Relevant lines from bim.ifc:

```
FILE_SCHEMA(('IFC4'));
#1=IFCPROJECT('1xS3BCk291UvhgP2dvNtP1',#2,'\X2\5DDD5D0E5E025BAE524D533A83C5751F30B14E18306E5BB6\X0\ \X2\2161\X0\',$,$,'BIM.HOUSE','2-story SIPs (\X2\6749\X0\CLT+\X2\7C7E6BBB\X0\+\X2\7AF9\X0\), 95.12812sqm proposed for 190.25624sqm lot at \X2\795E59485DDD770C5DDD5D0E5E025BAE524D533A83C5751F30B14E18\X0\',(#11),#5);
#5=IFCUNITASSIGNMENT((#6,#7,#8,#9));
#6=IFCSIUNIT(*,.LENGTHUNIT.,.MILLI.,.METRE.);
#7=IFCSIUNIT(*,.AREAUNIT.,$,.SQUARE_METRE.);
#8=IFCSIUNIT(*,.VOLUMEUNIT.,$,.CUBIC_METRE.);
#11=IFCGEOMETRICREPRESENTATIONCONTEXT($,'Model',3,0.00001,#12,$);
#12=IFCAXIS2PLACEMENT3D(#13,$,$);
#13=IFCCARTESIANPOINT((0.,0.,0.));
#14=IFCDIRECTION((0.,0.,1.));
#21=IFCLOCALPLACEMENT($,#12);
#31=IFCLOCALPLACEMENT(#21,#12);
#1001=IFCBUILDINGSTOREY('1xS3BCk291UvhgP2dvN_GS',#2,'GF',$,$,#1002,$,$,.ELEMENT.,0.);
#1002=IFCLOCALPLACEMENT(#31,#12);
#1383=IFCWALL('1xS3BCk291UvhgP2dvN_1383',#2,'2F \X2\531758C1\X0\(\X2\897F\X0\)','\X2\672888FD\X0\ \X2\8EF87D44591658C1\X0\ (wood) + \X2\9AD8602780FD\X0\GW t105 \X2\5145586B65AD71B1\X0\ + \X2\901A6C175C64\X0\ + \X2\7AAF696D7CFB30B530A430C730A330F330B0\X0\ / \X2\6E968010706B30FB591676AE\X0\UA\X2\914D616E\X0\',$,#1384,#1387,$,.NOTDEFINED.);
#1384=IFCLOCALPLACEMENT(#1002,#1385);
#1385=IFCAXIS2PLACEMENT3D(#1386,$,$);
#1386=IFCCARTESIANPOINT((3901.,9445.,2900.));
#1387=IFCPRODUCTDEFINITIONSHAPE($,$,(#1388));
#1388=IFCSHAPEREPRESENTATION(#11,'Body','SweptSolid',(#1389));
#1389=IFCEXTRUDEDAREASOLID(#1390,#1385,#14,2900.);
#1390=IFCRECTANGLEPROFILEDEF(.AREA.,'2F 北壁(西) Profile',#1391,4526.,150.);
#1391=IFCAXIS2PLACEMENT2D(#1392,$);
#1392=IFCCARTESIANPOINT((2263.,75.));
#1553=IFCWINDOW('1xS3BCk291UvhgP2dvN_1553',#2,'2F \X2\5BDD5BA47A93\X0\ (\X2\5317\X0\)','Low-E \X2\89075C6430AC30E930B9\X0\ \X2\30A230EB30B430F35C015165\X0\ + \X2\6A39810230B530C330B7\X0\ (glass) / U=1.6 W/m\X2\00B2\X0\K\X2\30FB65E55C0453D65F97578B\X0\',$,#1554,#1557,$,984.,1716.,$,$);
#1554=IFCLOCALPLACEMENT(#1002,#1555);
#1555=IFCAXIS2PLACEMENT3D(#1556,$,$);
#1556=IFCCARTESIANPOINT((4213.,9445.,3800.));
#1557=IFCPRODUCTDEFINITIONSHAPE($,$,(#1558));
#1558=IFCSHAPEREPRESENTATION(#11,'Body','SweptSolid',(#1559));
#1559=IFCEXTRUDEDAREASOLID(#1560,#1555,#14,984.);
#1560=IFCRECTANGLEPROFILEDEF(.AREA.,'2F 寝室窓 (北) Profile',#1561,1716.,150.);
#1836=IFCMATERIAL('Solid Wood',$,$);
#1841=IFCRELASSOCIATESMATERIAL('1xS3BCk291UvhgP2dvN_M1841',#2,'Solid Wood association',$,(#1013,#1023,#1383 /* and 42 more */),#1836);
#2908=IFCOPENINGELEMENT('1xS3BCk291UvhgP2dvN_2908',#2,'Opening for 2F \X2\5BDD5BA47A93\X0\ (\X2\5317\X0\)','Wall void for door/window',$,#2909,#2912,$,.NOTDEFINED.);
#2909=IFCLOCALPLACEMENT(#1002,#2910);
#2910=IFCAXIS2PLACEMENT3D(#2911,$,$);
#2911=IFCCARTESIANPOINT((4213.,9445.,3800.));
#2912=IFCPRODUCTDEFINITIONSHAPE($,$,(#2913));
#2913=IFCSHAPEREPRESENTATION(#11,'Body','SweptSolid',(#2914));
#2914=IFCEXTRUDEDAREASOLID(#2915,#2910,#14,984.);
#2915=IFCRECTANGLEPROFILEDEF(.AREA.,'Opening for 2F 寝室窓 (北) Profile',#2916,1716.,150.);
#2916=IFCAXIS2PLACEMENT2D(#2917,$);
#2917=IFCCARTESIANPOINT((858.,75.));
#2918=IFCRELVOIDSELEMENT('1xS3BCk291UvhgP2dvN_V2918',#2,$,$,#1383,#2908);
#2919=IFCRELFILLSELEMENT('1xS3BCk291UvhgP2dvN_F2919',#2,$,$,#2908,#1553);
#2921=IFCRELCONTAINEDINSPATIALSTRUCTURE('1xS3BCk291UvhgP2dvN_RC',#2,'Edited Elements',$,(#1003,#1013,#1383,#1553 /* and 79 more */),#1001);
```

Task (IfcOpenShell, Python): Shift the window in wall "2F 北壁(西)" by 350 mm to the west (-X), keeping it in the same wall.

```python
import ifcopenshell
import ifcopenshell.api.geometry
import ifcopenshell.util.placement

model = ifcopenshell.open("bim.ifc")

window = model.by_guid("1xS3BCk291UvhgP2dvN_1553")
opening = window.FillsVoids[0].RelatingOpeningElement
wall = opening.VoidsElements[0].RelatingBuildingElement

wall_matrix = ifcopenshell.util.placement.get_local_placement(wall.ObjectPlacement)
shift = wall_matrix[:3, 0] * -350.0
before = ifcopenshell.util.placement.get_local_placement(window.ObjectPlacement)[:3, 3].copy()

# The window is not placed relative to its opening, so move both.
for product in (opening, window):
    matrix = ifcopenshell.util.placement.get_local_placement(product.ObjectPlacement)
    matrix[:3, 3] += shift
    ifcopenshell.api.geometry.edit_object_placement(model, product=product, matrix=matrix, is_si=False)

after = ifcopenshell.util.placement.get_local_placement(window.ObjectPlacement)[:3, 3]
print("window moved by", (after - before).round(3) + 0.0)

model.write("bim_updated.ifc")
```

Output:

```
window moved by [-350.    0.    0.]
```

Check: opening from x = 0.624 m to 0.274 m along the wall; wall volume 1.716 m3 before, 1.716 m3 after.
